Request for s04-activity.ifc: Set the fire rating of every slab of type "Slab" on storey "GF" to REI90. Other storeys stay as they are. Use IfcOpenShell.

First a look at what the model holds.

```python
import ifcopenshell
import ifcopenshell.util.element

model = ifcopenshell.open("s04-activity.ifc")
print(model.schema)
storey = next(s for s in model.by_type("IfcBuildingStorey") if s.Name == "GF")
slabs = [e for e in ifcopenshell.util.element.get_decomposition(storey) if e.is_a("IfcSlab")]
seen = {}
for e in slabs:
    element_type = ifcopenshell.util.element.get_type(e)
    key = (element_type.Name if element_type != e and element_type else None, ifcopenshell.util.element.get_pset(e, "Pset_SlabCommon", "FireRating"))
    seen[key] = seen.get(key, 0) + 1
for (name, value), count in sorted(seen.items(), key=str):
    print(count, "x", name, "|", value)
```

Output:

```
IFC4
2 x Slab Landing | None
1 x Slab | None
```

```python
import ifcopenshell
import ifcopenshell.api.pset
import ifcopenshell.util.element

model = ifcopenshell.open("s04-activity.ifc")

storey = next(s for s in model.by_type("IfcBuildingStorey") if s.Name == "GF")
slabs = [e for e in ifcopenshell.util.element.get_decomposition(storey) if e.is_a("IfcSlab")]

count = 0
for e in slabs:
    element_type = ifcopenshell.util.element.get_type(e)
    if element_type in (None, e) or element_type.Name != "Slab":
        continue
    # add_pset returns the element's existing set when there is one.
    pset = ifcopenshell.api.pset.add_pset(model, product=e, name="Pset_SlabCommon")
    ifcopenshell.api.pset.edit_pset(model, pset=pset, properties={"FireRating": "REI90"})
    count += 1

print(count, "slabs updated")

model.write("s04-activity-out.ifc")
```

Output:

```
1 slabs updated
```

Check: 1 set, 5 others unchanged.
